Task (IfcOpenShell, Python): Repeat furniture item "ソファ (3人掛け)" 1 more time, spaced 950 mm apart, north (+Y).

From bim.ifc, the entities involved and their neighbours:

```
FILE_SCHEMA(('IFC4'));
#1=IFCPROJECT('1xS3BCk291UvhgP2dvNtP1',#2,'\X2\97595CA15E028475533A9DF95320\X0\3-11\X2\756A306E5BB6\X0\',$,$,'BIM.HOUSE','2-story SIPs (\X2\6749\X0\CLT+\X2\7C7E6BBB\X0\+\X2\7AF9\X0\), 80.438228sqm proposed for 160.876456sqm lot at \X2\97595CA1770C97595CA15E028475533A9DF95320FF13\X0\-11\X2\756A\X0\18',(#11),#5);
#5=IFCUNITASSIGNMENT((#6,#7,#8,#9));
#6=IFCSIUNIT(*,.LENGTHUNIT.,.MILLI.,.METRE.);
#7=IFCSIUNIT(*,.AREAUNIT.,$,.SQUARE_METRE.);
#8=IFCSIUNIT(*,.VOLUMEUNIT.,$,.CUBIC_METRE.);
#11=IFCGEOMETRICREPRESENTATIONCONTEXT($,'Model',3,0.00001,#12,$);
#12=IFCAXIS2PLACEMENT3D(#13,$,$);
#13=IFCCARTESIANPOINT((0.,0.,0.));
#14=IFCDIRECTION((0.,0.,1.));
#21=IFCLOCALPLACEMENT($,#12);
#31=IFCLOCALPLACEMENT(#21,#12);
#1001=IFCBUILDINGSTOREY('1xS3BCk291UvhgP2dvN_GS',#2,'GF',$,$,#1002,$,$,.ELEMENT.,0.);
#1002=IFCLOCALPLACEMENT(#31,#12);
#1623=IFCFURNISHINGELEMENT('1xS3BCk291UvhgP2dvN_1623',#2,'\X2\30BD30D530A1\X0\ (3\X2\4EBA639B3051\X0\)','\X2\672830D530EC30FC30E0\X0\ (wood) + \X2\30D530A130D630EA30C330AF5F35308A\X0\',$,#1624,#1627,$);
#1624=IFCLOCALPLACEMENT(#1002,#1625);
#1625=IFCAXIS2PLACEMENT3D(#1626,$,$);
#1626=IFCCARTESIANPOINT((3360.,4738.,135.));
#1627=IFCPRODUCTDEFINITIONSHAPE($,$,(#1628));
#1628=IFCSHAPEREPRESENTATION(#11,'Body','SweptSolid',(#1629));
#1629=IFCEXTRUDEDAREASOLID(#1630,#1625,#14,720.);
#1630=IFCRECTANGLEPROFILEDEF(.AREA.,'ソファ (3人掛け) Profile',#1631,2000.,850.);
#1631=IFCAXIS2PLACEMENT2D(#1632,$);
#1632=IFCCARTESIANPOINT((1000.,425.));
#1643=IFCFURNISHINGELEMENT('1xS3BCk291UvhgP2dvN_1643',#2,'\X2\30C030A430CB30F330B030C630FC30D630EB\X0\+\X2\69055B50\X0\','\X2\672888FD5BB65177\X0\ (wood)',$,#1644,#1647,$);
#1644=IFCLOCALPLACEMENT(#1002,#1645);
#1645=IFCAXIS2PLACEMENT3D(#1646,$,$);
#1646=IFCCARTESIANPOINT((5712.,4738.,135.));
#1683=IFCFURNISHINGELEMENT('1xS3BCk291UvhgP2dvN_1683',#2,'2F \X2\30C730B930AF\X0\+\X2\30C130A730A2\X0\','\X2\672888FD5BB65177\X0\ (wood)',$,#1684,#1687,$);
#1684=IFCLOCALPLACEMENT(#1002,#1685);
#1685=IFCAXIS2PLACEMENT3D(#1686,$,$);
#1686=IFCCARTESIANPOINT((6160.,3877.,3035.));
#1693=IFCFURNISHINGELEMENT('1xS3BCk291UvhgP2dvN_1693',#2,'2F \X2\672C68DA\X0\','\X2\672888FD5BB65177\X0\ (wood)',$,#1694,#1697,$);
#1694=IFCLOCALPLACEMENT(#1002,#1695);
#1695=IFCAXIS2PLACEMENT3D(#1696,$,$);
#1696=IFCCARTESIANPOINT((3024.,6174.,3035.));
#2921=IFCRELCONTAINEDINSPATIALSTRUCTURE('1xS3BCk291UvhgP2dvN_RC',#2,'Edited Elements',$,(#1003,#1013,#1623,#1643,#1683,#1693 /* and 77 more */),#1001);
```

```python
import numpy as np
import ifcopenshell
import ifcopenshell.api.geometry
import ifcopenshell.api.root
import ifcopenshell.util.element
import ifcopenshell.util.placement

model = ifcopenshell.open("bim.ifc")


def reuse_history(source, copy):
    """copy_class also copies each property set's owner history, people and application; keep the originals."""
    for rel in copy.IsDefinedBy:
        if rel.is_a("IfcRelDefinesByProperties") and (history := rel.RelatingPropertyDefinition.OwnerHistory):
            rel.RelatingPropertyDefinition.OwnerHistory = source.OwnerHistory
            ifcopenshell.util.element.remove_deep2(model, history)


source = model.by_guid("1xS3BCk291UvhgP2dvN_1623")
base = ifcopenshell.util.placement.get_local_placement(source.ObjectPlacement)
step = np.array([0.0, 1.0, 0.0]) * 950.0

for i in range(1, 2):
    copy = ifcopenshell.api.root.copy_class(model, product=source)
    copy.Representation = ifcopenshell.util.element.copy_deep(
        model, source.Representation, exclude=["IfcGeometricRepresentationContext", "IfcRepresentationMap"]
    )
    reuse_history(source, copy)
    matrix = base.copy()
    matrix[:3, 3] += i * step
    print("added at", matrix[:3, 3].round(3) + 0.0)
    ifcopenshell.api.geometry.edit_object_placement(model, product=copy, matrix=matrix, is_si=False)

model.write("bim_edited.ifc")
```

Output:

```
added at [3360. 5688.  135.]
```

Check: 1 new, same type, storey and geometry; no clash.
